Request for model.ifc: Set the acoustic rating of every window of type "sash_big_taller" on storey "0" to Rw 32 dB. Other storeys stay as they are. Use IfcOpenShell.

First a look at what the model holds.

```python
import ifcopenshell
import ifcopenshell.util.element

model = ifcopenshell.open("model.ifc")
print(model.schema)
storey = next(s for s in model.by_type("IfcBuildingStorey") if s.Name == "0")
windows = [e for e in ifcopenshell.util.element.get_decomposition(storey) if e.is_a("IfcWindow")]
seen = {}
for e in windows:
    element_type = ifcopenshell.util.element.get_type(e)
    key = (element_type.Name if element_type != e and element_type else None, ifcopenshell.util.element.get_pset(e, "Pset_WindowCommon", "AcousticRating"))
    seen[key] = seen.get(key, 0) + 1
for (name, value), count in sorted(seen.items(), key=str):
    print(count, "x", name, "|", value)
```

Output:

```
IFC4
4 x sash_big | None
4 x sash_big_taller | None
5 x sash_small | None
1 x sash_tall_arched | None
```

```python
import ifcopenshell
import ifcopenshell.api.pset
import ifcopenshell.util.element

model = ifcopenshell.open("model.ifc")

storey = next(s for s in model.by_type("IfcBuildingStorey") if s.Name == "0")
windows = [e for e in ifcopenshell.util.element.get_decomposition(storey) if e.is_a("IfcWindow")]

count = 0
for e in windows:
    element_type = ifcopenshell.util.element.get_type(e)
    if element_type in (None, e) or element_type.Name != "sash_big_taller":
        continue
    # add_pset returns the element's existing set when there is one.
    pset = ifcopenshell.api.pset.add_pset(model, product=e, name="Pset_WindowCommon")
    ifcopenshell.api.pset.edit_pset(model, pset=pset, properties={"AcousticRating": "Rw 32 dB"})
    count += 1

print(count, "windows updated")

model.write("model-out.ifc")
```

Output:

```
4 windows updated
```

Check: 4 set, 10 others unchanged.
